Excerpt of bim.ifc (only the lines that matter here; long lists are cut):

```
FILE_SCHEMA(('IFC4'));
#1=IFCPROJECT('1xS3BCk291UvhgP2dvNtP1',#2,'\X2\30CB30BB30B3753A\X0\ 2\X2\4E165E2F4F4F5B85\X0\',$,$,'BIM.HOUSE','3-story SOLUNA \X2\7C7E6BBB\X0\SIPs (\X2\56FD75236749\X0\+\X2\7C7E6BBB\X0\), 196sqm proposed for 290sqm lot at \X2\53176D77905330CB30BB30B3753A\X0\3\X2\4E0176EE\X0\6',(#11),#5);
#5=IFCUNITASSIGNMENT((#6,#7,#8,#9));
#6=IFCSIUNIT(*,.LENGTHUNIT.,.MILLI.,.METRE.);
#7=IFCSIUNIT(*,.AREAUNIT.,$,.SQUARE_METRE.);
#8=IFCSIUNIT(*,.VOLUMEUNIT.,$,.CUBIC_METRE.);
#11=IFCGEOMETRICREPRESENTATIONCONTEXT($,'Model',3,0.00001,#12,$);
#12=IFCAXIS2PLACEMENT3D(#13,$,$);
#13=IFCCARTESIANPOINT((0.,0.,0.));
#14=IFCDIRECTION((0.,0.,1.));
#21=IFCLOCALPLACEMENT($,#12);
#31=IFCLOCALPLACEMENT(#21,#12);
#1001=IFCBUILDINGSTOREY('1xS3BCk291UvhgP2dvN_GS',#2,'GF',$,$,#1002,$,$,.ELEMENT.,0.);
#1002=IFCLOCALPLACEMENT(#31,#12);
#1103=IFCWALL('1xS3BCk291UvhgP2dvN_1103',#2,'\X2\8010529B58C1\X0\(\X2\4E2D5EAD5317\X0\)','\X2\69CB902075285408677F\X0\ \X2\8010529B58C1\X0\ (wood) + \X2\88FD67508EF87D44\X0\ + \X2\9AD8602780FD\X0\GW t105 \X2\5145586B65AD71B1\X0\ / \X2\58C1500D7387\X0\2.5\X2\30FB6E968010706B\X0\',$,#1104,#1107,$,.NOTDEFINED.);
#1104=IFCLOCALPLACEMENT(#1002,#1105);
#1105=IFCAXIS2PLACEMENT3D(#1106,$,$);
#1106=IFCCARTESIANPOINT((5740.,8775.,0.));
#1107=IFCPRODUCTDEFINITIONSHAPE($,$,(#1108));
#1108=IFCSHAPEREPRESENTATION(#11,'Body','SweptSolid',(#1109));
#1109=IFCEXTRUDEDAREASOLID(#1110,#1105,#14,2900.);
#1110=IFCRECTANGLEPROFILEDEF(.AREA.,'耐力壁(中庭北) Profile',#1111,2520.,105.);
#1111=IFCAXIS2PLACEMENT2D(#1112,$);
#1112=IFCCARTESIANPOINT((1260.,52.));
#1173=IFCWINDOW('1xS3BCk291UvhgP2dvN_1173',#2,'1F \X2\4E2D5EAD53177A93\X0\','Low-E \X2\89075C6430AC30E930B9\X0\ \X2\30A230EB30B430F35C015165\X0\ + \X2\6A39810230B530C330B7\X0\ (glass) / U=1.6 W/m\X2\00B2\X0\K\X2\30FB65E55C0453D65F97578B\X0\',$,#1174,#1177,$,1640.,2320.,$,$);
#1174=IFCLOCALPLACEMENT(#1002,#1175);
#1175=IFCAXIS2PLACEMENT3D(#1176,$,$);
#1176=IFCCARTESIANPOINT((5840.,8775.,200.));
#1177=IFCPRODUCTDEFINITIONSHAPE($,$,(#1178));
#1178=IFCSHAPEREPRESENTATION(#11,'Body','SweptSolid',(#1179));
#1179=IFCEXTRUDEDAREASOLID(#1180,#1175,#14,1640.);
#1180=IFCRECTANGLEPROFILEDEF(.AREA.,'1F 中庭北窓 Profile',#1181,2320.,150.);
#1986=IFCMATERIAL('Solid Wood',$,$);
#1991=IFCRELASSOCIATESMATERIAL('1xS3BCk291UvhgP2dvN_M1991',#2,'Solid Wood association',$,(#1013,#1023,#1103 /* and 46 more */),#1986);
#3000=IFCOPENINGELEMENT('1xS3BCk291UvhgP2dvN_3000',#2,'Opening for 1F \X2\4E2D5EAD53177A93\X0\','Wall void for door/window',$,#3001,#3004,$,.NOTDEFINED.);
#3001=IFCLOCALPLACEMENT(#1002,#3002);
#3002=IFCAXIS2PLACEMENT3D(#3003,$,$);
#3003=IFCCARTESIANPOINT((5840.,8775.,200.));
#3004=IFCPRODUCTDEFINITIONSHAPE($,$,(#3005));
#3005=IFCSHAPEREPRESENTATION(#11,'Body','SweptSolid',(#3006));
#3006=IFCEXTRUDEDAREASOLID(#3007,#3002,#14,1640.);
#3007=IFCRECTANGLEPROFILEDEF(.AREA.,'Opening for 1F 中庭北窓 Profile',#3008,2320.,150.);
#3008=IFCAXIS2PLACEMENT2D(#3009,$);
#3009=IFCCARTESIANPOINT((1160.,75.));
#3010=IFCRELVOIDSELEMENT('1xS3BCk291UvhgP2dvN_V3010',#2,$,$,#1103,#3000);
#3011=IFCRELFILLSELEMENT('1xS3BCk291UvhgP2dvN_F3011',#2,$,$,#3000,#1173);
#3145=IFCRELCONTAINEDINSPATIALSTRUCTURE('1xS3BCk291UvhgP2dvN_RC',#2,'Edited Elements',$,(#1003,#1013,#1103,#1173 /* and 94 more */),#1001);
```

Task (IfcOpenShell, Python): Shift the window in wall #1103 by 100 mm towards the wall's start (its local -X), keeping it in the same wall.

```python
import ifcopenshell
import ifcopenshell.api.geometry
import ifcopenshell.util.placement

model = ifcopenshell.open("bim.ifc")

window = model.by_guid("1xS3BCk291UvhgP2dvN_1173")
opening = window.FillsVoids[0].RelatingOpeningElement
wall = opening.VoidsElements[0].RelatingBuildingElement

wall_matrix = ifcopenshell.util.placement.get_local_placement(wall.ObjectPlacement)
shift = wall_matrix[:3, 0] * -100.0
before = ifcopenshell.util.placement.get_local_placement(window.ObjectPlacement)[:3, 3].copy()

# The window is not placed relative to its opening, so move both.
for product in (opening, window):
    matrix = ifcopenshell.util.placement.get_local_placement(product.ObjectPlacement)
    matrix[:3, 3] += shift
    ifcopenshell.api.geometry.edit_object_placement(model, product=product, matrix=matrix, is_si=False)

after = ifcopenshell.util.placement.get_local_placement(window.ObjectPlacement)[:3, 3]
print("window moved by", (after - before).round(3) + 0.0)

model.write("bim_v2.ifc")
```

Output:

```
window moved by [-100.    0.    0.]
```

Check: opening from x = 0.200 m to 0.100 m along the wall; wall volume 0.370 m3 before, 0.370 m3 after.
